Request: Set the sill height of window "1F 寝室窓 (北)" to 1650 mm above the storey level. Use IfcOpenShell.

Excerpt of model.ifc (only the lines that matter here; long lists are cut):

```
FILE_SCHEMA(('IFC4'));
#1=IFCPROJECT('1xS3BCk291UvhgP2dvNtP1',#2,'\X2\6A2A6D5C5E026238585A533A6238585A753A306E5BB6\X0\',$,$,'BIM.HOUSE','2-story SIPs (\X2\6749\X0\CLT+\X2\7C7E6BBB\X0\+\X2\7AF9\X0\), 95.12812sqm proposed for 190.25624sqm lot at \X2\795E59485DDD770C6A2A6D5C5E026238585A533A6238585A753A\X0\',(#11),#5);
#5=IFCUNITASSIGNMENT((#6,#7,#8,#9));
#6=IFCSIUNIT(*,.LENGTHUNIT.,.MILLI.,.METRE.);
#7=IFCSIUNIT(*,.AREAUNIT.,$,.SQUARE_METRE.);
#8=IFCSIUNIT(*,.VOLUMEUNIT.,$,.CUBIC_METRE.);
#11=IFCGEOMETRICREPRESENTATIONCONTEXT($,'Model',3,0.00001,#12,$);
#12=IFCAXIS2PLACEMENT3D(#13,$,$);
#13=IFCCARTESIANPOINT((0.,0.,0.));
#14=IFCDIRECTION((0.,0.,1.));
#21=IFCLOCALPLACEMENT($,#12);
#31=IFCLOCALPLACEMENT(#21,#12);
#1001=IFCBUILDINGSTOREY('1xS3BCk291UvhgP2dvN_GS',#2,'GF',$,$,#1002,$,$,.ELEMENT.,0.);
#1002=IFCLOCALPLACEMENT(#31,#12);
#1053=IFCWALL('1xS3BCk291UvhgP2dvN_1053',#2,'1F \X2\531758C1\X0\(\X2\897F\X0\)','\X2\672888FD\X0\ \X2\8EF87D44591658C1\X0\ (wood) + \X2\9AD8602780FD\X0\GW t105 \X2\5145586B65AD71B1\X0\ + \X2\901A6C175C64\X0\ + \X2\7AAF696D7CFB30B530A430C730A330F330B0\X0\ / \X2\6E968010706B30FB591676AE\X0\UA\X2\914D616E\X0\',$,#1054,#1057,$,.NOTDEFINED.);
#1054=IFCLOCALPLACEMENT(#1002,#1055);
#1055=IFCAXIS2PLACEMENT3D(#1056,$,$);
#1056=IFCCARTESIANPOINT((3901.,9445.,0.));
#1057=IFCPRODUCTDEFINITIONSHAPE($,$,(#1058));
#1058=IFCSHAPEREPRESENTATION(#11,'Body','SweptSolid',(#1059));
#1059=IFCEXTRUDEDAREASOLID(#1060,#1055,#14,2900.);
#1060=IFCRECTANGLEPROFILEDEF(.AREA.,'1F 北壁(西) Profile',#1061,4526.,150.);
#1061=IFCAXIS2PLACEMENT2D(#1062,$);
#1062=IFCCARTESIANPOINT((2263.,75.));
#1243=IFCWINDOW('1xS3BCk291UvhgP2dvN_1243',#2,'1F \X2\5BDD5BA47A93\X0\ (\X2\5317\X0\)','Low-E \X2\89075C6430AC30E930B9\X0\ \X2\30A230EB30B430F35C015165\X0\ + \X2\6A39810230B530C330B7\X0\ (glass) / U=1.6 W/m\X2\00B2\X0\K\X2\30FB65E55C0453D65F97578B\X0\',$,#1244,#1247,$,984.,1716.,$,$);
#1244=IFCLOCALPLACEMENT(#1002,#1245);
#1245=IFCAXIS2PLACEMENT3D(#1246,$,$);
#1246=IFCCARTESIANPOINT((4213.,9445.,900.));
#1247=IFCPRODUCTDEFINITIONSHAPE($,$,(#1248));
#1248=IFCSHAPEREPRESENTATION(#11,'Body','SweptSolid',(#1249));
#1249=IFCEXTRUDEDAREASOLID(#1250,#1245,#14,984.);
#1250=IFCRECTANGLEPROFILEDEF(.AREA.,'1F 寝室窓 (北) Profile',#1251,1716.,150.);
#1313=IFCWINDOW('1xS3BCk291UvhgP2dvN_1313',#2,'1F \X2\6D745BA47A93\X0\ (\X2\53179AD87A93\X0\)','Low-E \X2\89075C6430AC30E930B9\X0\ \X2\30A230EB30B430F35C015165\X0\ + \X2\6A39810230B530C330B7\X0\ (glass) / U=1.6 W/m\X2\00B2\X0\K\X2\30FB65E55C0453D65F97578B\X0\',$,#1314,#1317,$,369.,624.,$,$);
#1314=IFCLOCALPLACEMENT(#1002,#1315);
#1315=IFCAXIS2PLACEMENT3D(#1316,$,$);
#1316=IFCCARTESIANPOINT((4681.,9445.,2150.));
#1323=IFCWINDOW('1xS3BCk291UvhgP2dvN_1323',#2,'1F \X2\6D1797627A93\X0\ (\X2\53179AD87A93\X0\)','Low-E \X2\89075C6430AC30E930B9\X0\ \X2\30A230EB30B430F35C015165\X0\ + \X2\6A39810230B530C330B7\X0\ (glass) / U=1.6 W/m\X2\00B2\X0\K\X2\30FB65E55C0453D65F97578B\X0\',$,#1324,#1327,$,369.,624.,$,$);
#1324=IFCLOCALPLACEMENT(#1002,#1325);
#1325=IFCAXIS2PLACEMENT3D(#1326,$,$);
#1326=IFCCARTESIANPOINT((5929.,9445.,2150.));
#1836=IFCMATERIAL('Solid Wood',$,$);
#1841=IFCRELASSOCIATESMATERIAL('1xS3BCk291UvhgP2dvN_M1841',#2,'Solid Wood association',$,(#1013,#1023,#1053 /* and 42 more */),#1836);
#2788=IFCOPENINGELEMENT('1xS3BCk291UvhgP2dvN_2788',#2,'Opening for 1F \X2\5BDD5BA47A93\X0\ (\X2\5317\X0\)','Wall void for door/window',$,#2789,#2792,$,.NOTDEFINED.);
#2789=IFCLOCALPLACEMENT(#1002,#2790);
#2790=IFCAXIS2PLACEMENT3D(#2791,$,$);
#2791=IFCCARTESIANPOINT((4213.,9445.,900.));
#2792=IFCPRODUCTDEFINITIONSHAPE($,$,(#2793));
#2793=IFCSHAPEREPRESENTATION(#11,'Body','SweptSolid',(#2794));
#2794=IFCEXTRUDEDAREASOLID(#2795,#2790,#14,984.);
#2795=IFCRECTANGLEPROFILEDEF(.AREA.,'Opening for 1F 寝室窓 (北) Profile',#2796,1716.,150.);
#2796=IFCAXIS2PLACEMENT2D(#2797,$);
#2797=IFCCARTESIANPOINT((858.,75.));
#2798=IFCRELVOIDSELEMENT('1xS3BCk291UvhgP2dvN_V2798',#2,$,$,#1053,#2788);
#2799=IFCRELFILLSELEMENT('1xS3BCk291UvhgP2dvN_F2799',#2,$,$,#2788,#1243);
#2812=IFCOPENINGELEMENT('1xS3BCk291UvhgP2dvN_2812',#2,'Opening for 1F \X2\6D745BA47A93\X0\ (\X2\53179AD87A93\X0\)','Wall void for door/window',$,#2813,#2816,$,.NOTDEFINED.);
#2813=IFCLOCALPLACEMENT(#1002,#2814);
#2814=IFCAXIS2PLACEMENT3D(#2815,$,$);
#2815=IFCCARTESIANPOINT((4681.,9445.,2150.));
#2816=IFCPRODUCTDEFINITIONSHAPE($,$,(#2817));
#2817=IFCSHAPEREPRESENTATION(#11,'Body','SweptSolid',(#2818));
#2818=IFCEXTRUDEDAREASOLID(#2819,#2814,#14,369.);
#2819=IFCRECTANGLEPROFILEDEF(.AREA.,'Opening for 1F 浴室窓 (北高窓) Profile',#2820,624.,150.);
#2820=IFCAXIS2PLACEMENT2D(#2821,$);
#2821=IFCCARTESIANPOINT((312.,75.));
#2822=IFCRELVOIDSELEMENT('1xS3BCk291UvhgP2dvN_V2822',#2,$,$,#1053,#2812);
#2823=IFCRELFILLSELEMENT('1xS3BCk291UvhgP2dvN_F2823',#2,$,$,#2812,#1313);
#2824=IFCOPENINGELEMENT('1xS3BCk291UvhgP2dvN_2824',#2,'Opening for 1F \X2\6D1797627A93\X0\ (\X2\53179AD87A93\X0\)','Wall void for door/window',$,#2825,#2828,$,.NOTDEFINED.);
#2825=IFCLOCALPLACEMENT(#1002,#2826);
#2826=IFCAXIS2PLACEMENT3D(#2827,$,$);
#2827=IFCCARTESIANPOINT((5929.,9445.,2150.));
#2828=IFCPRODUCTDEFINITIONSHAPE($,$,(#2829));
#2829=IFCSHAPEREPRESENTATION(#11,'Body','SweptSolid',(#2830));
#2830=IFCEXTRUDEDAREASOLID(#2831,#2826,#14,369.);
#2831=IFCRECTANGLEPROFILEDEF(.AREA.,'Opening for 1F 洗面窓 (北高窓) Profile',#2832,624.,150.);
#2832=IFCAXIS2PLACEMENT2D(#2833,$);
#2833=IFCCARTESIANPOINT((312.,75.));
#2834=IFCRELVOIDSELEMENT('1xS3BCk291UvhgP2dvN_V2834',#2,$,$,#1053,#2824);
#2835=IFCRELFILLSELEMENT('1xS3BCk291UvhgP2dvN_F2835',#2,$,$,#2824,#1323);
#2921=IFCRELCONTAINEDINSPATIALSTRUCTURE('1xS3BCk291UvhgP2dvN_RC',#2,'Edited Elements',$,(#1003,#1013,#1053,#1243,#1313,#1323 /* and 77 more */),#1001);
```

```python
import numpy as np
import ifcopenshell
import ifcopenshell.api.geometry
import ifcopenshell.geom
import ifcopenshell.util.element
import ifcopenshell.util.placement
import ifcopenshell.util.shape
import ifcopenshell.util.unit

model = ifcopenshell.open("model.ifc")
unit_scale = ifcopenshell.util.unit.calculate_unit_scale(model)

window = model.by_guid("1xS3BCk291UvhgP2dvN_1243")
opening = window.FillsVoids[0].RelatingOpeningElement
storey = ifcopenshell.util.element.get_container(window, ifc_class="IfcBuildingStorey")
level = ifcopenshell.util.placement.get_local_placement(storey.ObjectPlacement)[2, 3]

# The opening's origin need not be at the sill, so measure its lowest point.
shape = ifcopenshell.geom.create_shape(ifcopenshell.geom.settings(), opening)
bottom = ifcopenshell.util.shape.get_shape_bottom_elevation(shape, shape.geometry) / unit_scale
dz = level + 1.65 / unit_scale - bottom

shift = np.array([0.0, 0.0, dz])
# The window is not placed relative to its opening, so move both.
for product in (opening, window):
    matrix = ifcopenshell.util.placement.get_local_placement(product.ObjectPlacement)
    matrix[:3, 3] += shift
    ifcopenshell.api.geometry.edit_object_placement(model, product=product, matrix=matrix, is_si=False)

print(f"moved by {dz * unit_scale:+.3f} m")

model.write("model-out.ifc")
```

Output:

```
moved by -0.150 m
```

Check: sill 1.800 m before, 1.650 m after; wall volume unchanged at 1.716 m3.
